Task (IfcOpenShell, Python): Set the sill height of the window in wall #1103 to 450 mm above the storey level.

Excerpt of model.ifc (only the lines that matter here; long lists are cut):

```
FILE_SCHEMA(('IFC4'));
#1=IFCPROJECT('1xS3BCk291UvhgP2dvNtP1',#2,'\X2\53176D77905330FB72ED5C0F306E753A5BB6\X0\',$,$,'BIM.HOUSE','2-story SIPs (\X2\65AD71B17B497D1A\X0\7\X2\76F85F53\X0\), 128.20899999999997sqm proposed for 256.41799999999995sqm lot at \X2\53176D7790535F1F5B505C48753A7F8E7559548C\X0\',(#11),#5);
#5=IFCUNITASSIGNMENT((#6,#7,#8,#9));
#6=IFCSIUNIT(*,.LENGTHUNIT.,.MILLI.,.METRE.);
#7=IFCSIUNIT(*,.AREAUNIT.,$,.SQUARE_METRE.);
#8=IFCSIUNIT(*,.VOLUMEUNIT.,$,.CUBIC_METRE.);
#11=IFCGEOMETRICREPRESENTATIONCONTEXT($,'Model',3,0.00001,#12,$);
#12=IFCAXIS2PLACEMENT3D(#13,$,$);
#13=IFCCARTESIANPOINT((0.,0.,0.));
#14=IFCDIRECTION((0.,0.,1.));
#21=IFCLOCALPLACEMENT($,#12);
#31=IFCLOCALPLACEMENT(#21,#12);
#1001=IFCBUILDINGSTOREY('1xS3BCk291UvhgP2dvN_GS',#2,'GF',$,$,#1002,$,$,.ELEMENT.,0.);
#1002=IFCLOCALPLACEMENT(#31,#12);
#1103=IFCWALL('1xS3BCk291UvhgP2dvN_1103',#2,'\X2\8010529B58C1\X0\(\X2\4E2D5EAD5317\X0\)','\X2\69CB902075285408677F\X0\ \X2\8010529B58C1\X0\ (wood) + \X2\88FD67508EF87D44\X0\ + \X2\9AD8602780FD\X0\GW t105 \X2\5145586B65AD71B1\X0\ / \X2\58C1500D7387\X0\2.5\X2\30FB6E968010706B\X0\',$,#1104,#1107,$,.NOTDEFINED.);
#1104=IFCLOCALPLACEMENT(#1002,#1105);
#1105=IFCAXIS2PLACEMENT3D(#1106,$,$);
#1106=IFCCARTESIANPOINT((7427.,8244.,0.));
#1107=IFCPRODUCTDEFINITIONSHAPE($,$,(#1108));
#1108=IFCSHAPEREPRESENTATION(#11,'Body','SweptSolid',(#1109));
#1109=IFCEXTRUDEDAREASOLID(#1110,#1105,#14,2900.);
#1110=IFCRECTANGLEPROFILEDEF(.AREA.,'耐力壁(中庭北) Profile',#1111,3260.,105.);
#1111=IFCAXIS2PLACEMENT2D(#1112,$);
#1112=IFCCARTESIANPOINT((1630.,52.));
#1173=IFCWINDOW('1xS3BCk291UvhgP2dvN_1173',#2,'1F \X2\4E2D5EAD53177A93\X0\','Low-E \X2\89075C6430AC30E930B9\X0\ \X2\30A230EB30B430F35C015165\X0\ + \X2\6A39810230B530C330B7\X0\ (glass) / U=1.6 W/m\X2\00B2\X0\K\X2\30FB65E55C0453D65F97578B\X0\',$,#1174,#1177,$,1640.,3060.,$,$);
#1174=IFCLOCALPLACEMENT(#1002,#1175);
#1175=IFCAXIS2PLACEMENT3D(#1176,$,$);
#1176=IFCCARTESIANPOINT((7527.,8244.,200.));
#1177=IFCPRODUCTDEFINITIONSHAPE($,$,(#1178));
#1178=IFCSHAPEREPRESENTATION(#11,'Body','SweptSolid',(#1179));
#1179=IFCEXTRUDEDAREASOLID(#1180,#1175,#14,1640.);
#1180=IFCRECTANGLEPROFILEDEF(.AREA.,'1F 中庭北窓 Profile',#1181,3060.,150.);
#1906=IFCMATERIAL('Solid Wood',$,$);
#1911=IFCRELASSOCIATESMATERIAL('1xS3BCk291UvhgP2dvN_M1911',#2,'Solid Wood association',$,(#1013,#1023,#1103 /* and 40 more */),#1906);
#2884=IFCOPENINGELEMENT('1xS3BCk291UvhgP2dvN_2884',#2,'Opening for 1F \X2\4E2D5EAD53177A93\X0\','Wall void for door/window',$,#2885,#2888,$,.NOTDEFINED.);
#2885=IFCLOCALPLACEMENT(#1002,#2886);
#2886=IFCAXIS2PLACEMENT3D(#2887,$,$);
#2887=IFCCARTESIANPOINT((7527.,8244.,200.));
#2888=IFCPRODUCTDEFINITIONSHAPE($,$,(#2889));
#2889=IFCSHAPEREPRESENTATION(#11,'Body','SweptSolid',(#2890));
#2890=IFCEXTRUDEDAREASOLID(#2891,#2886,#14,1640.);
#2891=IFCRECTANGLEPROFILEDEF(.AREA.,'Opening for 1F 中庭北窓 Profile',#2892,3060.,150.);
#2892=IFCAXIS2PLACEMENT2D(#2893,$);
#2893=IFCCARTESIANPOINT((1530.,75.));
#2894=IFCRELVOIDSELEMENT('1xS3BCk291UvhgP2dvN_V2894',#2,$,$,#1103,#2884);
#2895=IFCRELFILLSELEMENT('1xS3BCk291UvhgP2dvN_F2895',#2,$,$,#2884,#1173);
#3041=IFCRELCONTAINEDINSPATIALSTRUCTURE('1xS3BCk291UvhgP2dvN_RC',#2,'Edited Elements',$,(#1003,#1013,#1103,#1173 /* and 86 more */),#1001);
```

```python
import numpy as np
import ifcopenshell
import ifcopenshell.api.geometry
import ifcopenshell.geom
import ifcopenshell.util.element
import ifcopenshell.util.placement
import ifcopenshell.util.shape
import ifcopenshell.util.unit

model = ifcopenshell.open("model.ifc")
unit_scale = ifcopenshell.util.unit.calculate_unit_scale(model)

window = model.by_id(1173)
opening = window.FillsVoids[0].RelatingOpeningElement
storey = ifcopenshell.util.element.get_container(window, ifc_class="IfcBuildingStorey")
level = ifcopenshell.util.placement.get_local_placement(storey.ObjectPlacement)[2, 3]

# The opening's origin need not be at the sill, so measure its lowest point.
shape = ifcopenshell.geom.create_shape(ifcopenshell.geom.settings(), opening)
bottom = ifcopenshell.util.shape.get_shape_bottom_elevation(shape, shape.geometry) / unit_scale
dz = level + 0.45 / unit_scale - bottom

shift = np.array([0.0, 0.0, dz])
# The window is not placed relative to its opening, so move both.
for product in (opening, window):
    matrix = ifcopenshell.util.placement.get_local_placement(product.ObjectPlacement)
    matrix[:3, 3] += shift
    ifcopenshell.api.geometry.edit_object_placement(model, product=product, matrix=matrix, is_si=False)

print(f"moved by {dz * unit_scale:+.3f} m")

model.write("model_v2.ifc")
```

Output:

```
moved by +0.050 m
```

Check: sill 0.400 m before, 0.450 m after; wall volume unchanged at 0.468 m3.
